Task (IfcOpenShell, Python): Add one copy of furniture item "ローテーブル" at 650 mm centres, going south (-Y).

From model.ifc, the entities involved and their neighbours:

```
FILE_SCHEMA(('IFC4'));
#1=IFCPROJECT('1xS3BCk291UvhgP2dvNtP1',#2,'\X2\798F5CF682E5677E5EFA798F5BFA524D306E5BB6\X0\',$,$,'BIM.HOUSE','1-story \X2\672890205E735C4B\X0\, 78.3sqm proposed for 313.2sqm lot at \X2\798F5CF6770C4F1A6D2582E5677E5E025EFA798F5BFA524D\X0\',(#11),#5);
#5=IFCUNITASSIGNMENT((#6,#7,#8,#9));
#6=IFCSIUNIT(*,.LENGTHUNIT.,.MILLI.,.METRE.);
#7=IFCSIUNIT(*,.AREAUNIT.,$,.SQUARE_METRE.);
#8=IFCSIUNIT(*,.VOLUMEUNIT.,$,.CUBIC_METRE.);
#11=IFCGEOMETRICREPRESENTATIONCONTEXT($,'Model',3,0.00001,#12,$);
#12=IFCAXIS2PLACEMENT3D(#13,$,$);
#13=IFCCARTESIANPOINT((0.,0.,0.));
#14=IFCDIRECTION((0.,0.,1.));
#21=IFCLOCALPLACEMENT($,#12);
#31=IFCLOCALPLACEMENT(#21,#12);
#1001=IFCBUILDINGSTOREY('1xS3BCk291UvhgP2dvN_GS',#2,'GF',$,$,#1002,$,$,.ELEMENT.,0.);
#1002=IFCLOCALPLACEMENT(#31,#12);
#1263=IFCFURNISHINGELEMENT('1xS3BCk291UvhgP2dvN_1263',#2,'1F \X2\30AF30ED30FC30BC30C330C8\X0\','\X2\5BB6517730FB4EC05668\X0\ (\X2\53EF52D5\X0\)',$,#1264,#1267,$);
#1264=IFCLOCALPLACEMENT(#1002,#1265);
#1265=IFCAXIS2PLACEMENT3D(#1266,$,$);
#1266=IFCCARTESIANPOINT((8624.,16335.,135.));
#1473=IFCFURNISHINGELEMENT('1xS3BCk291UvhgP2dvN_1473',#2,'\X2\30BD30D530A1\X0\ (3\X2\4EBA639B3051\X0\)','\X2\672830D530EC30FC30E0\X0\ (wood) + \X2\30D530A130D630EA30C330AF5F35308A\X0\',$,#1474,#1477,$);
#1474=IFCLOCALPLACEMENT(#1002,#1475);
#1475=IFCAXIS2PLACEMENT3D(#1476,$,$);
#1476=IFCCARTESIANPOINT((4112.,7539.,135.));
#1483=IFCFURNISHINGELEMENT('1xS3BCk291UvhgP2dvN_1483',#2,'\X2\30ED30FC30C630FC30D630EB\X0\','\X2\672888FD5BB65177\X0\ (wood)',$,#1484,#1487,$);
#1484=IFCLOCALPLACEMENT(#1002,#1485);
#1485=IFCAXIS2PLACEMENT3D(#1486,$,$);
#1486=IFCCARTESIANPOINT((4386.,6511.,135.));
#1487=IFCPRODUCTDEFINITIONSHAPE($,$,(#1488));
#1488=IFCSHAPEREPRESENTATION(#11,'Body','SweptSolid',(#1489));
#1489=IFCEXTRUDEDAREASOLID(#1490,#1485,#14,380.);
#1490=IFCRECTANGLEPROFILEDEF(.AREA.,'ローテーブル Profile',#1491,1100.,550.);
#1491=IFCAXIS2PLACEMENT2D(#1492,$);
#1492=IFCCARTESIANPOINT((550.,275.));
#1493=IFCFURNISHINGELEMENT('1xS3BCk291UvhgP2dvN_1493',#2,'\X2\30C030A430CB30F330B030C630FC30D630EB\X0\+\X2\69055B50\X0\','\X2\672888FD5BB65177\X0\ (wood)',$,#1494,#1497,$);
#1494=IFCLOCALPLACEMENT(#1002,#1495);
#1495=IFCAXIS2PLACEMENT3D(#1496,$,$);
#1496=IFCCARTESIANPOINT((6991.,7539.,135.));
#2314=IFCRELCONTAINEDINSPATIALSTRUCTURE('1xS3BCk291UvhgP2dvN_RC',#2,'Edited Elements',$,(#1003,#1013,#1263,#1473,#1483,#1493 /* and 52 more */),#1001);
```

```python
import numpy as np
import ifcopenshell
import ifcopenshell.api.geometry
import ifcopenshell.api.root
import ifcopenshell.util.element
import ifcopenshell.util.placement

model = ifcopenshell.open("model.ifc")


def reuse_history(source, copy):
    """copy_class also copies each property set's owner history, people and application; keep the originals."""
    for rel in copy.IsDefinedBy:
        if rel.is_a("IfcRelDefinesByProperties") and (history := rel.RelatingPropertyDefinition.OwnerHistory):
            rel.RelatingPropertyDefinition.OwnerHistory = source.OwnerHistory
            ifcopenshell.util.element.remove_deep2(model, history)


source = model.by_guid("1xS3BCk291UvhgP2dvN_1483")
base = ifcopenshell.util.placement.get_local_placement(source.ObjectPlacement)
step = np.array([0.0, -1.0, 0.0]) * 650.0

for i in range(1, 2):
    copy = ifcopenshell.api.root.copy_class(model, product=source)
    copy.Representation = ifcopenshell.util.element.copy_deep(
        model, source.Representation, exclude=["IfcGeometricRepresentationContext", "IfcRepresentationMap"]
    )
    reuse_history(source, copy)
    matrix = base.copy()
    matrix[:3, 3] += i * step
    print("added at", matrix[:3, 3].round(3) + 0.0)
    ifcopenshell.api.geometry.edit_object_placement(model, product=copy, matrix=matrix, is_si=False)

model.write("model_updated.ifc")
```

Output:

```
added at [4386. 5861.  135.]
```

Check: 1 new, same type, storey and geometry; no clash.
